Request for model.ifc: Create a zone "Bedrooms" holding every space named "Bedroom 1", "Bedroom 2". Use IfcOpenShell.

First a look at what the model holds.

```python
import ifcopenshell

model = ifcopenshell.open("model.ifc")
print(model.schema)
seen = {}
for space in model.by_type("IfcSpace"):
    seen[space.LongName] = seen.get(space.LongName, 0) + 1
for name, count in sorted(seen.items(), key=str):
    print(count, "x", name)
print("zones:", [z.Name for z in model.by_type("IfcZone")][:20])
```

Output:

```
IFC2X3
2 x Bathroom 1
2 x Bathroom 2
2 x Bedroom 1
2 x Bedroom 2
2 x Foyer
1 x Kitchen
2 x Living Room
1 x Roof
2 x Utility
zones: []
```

```python
import ifcopenshell
import ifcopenshell.api.group
import ifcopenshell.api.root

model = ifcopenshell.open("model.ifc")

names = {"Bedroom 1", "Bedroom 2"}
spaces = [s for s in model.by_type("IfcSpace") if s.LongName in names]

zone = ifcopenshell.api.root.create_entity(model, ifc_class="IfcZone", name="Bedrooms")
ifcopenshell.api.group.assign_group(model, products=spaces, group=zone)
print(len(spaces), "spaces in", zone.Name)

model.write("model_edited.ifc")
```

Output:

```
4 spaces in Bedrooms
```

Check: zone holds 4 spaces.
